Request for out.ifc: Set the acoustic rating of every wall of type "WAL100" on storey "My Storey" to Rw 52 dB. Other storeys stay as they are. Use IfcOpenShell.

First a look at what the model holds.

```python
import ifcopenshell
import ifcopenshell.util.element

model = ifcopenshell.open("out.ifc")
print(model.schema)
storey = next(s for s in model.by_type("IfcBuildingStorey") if s.Name == "My Storey")
walls = [e for e in ifcopenshell.util.element.get_decomposition(storey) if e.is_a("IfcWall")]
seen = {}
for e in walls:
    element_type = ifcopenshell.util.element.get_type(e)
    key = (element_type.Name if element_type != e and element_type else None, ifcopenshell.util.element.get_pset(e, "Pset_WallCommon", "AcousticRating"))
    seen[key] = seen.get(key, 0) + 1
for (name, value), count in sorted(seen.items(), key=str):
    print(count, "x", name, "|", value)
```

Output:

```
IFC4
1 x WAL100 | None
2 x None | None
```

```python
import ifcopenshell
import ifcopenshell.api.pset
import ifcopenshell.util.element

model = ifcopenshell.open("out.ifc")

storey = next(s for s in model.by_type("IfcBuildingStorey") if s.Name == "My Storey")
walls = [e for e in ifcopenshell.util.element.get_decomposition(storey) if e.is_a("IfcWall")]

count = 0
for e in walls:
    element_type = ifcopenshell.util.element.get_type(e)
    if element_type in (None, e) or element_type.Name != "WAL100":
        continue
    # add_pset returns the element's existing set when there is one.
    pset = ifcopenshell.api.pset.add_pset(model, product=e, name="Pset_WallCommon")
    ifcopenshell.api.pset.edit_pset(model, pset=pset, properties={"AcousticRating": "Rw 52 dB"})
    count += 1

print(count, "walls updated")

model.write("out-out.ifc")
```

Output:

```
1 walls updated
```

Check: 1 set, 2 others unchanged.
